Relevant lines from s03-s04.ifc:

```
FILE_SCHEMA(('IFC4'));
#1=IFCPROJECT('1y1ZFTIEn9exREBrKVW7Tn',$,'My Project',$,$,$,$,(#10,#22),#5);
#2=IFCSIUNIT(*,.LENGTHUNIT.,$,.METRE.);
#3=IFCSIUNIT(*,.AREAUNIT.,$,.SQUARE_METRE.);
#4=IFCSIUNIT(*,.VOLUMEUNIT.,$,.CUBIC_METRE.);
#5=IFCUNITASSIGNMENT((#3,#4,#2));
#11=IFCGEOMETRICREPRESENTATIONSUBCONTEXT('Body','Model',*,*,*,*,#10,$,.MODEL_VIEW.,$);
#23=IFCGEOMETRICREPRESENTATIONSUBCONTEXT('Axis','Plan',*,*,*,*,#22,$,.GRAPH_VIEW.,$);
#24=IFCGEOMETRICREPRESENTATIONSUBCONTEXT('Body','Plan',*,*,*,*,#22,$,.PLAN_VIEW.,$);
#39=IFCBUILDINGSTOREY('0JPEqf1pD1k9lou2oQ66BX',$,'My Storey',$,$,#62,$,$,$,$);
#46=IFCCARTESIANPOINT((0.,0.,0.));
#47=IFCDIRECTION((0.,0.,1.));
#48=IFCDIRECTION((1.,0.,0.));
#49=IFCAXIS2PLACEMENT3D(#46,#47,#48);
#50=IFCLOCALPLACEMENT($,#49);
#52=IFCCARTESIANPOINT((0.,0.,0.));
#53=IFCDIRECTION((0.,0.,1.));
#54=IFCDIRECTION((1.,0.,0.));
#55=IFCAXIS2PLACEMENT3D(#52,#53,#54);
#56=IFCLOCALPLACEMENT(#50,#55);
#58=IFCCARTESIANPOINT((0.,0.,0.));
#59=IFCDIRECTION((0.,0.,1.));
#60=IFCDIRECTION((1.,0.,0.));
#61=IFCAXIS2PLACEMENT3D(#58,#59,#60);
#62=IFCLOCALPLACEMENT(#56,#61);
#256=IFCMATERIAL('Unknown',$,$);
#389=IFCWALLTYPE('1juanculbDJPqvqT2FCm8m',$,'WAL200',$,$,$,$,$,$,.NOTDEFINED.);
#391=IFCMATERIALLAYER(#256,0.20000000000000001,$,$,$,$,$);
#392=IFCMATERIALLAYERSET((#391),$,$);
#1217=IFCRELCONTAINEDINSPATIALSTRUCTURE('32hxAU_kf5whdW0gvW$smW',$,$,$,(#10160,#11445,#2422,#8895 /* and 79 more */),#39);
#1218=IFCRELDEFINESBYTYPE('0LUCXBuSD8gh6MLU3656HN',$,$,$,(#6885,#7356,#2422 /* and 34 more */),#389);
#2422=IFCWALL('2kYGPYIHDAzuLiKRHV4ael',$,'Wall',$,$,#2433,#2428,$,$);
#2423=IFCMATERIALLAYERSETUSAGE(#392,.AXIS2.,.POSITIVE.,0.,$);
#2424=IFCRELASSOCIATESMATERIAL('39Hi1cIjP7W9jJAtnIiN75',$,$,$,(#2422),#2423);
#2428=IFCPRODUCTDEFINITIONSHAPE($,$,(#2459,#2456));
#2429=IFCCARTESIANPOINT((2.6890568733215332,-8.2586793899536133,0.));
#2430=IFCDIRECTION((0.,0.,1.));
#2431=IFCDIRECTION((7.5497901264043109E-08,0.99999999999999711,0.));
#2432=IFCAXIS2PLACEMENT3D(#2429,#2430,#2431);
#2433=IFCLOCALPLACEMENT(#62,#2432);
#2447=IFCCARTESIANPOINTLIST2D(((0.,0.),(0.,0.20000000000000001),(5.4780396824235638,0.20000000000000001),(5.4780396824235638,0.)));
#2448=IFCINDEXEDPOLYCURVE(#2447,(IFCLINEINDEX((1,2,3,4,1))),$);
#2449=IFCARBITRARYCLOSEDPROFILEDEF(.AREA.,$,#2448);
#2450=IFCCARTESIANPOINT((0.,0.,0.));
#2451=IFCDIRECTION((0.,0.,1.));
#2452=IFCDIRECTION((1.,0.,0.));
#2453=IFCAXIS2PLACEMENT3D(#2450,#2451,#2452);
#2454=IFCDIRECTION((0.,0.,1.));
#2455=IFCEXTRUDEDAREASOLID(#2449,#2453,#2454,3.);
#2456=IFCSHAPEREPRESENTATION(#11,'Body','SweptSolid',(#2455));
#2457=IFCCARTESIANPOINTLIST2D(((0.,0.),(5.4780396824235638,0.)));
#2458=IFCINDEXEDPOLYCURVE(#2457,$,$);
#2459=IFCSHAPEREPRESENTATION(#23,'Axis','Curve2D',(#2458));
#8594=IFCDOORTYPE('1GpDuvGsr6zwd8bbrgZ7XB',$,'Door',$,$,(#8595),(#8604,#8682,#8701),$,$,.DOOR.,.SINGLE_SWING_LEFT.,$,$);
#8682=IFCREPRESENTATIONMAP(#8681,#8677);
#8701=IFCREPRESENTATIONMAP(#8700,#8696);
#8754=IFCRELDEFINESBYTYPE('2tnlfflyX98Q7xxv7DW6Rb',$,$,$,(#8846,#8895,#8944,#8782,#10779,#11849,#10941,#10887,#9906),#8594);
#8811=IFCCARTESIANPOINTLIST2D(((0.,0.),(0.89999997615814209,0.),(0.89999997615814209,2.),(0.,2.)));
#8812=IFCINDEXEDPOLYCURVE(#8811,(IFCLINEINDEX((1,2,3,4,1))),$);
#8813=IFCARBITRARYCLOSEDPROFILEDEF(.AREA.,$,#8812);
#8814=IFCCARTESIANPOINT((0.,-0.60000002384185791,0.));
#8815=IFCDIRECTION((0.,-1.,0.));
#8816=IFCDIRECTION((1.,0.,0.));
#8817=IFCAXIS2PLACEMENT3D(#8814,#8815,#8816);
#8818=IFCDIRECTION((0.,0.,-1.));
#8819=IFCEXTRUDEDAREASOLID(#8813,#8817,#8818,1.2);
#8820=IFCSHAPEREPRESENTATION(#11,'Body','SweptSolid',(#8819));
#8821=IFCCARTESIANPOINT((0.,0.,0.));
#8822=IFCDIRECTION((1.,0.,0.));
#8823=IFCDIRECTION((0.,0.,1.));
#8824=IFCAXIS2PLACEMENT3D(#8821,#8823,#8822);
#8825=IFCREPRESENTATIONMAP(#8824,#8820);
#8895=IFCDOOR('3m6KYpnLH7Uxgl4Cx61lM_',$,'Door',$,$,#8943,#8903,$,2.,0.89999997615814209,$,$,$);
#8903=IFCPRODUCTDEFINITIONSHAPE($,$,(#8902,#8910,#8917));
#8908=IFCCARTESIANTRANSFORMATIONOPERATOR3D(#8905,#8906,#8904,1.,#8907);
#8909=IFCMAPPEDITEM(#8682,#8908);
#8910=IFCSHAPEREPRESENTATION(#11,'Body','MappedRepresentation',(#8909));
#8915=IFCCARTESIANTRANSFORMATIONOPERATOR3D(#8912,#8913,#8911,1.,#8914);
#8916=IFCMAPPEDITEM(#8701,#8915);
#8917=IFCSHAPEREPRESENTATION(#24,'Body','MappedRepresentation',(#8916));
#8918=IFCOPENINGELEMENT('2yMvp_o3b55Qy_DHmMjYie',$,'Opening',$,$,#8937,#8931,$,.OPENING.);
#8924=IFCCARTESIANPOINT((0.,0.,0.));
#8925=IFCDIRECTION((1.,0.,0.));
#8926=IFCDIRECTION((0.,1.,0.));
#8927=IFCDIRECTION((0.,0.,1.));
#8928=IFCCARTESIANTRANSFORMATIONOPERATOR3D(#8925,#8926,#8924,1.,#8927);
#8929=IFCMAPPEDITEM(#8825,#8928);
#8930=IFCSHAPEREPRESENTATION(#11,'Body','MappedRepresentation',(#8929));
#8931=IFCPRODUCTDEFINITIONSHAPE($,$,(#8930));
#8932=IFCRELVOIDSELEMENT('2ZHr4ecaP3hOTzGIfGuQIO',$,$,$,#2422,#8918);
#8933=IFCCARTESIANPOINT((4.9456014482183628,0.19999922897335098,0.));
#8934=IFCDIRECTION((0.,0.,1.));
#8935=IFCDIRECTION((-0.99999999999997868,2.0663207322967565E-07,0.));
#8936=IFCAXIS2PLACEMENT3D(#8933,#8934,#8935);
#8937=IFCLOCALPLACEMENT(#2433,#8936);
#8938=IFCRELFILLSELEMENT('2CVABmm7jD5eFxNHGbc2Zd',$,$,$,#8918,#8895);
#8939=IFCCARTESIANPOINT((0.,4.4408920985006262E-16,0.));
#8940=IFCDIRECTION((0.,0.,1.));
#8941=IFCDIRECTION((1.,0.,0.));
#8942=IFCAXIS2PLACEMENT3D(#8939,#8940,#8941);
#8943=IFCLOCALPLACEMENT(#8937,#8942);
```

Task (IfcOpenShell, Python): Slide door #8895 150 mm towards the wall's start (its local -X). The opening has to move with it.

```python
import ifcopenshell
import ifcopenshell.api.geometry
import ifcopenshell.util.placement

model = ifcopenshell.open("s03-s04.ifc")

door = model.by_guid("3m6KYpnLH7Uxgl4Cx61lM_")
opening = door.FillsVoids[0].RelatingOpeningElement
wall = opening.VoidsElements[0].RelatingBuildingElement

wall_matrix = ifcopenshell.util.placement.get_local_placement(wall.ObjectPlacement)
shift = wall_matrix[:3, 0] * -0.15
before = ifcopenshell.util.placement.get_local_placement(door.ObjectPlacement)[:3, 3].copy()

# The door is placed relative to its opening, so it follows when the opening moves.
matrix = ifcopenshell.util.placement.get_local_placement(opening.ObjectPlacement)
matrix[:3, 3] += shift
ifcopenshell.api.geometry.edit_object_placement(
    model, product=opening, matrix=matrix, is_si=False, should_transform_children=True
)

after = ifcopenshell.util.placement.get_local_placement(door.ObjectPlacement)[:3, 3]
print("door moved by", (after - before).round(3) + 0.0)

model.write("s03-s04-out.ifc")
```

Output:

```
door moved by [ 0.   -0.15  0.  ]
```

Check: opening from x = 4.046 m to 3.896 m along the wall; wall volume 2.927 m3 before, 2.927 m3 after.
